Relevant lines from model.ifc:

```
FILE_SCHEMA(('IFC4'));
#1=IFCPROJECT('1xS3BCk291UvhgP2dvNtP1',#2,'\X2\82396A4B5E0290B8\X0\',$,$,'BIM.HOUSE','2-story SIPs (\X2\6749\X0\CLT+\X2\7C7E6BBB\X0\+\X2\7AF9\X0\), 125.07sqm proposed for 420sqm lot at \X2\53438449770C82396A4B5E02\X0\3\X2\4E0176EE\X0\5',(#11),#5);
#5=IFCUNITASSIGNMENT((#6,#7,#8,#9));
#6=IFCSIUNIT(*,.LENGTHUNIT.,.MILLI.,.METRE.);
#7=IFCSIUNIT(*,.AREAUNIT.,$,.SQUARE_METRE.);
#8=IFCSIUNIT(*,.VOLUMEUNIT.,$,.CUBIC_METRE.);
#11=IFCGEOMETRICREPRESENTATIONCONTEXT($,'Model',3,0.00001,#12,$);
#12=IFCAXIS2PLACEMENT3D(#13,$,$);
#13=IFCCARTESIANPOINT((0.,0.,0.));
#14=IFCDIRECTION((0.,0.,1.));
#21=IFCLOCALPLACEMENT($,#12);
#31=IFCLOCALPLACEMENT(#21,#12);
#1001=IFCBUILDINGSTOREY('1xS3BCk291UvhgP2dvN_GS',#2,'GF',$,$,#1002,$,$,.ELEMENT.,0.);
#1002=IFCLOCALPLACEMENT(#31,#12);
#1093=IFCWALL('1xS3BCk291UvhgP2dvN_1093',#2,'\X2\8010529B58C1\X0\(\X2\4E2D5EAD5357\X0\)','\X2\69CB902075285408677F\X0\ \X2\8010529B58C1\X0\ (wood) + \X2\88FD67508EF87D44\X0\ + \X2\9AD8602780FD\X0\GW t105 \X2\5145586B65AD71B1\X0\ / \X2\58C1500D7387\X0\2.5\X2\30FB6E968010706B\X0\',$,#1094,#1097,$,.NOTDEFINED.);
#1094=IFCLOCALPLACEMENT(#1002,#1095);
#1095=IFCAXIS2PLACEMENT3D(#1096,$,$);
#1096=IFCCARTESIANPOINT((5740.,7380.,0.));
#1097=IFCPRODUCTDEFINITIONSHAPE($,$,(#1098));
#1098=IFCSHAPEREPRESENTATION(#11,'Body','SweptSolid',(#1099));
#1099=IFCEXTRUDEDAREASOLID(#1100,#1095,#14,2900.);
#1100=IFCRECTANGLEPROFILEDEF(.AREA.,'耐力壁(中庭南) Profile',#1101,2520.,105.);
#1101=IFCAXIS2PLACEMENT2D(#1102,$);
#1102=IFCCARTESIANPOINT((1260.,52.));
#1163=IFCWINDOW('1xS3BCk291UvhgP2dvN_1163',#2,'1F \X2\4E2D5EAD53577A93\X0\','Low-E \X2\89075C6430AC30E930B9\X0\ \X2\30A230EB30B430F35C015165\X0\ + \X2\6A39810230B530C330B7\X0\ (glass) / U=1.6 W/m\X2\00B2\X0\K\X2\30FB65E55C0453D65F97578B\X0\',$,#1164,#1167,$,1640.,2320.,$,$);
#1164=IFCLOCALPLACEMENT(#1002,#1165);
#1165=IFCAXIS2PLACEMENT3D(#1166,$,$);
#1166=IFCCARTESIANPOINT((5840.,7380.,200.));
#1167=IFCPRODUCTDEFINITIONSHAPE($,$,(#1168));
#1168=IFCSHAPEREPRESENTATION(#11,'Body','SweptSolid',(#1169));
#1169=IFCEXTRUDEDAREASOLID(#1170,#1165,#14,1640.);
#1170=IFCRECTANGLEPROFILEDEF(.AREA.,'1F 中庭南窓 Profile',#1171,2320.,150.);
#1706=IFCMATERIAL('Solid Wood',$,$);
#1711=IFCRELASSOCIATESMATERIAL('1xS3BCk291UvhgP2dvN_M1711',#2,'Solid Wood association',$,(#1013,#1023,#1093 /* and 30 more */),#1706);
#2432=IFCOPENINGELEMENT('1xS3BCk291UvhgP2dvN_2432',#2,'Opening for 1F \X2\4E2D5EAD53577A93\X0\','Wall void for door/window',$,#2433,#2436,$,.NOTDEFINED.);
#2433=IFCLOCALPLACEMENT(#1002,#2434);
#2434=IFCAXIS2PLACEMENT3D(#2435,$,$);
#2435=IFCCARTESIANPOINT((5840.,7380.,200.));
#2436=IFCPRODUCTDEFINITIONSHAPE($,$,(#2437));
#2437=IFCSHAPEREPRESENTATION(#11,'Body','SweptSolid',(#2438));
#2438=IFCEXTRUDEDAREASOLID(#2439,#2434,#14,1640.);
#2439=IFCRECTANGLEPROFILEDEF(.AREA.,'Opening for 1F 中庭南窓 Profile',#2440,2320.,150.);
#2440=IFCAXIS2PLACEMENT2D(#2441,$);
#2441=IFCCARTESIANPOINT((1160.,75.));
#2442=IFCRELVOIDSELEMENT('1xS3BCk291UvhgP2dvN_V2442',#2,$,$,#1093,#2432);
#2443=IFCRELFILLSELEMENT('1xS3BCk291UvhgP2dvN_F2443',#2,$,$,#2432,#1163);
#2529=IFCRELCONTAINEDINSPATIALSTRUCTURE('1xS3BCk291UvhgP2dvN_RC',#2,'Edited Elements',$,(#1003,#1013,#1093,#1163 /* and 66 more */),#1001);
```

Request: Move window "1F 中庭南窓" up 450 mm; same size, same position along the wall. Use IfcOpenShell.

```python
import numpy as np
import ifcopenshell
import ifcopenshell.api.geometry
import ifcopenshell.util.placement
import ifcopenshell.util.unit

model = ifcopenshell.open("model.ifc")
unit_scale = ifcopenshell.util.unit.calculate_unit_scale(model)

window = model.by_guid("1xS3BCk291UvhgP2dvN_1163")
opening = window.FillsVoids[0].RelatingOpeningElement
dz = 0.45 / unit_scale

shift = np.array([0.0, 0.0, dz])
# The window is not placed relative to its opening, so move both.
for product in (opening, window):
    matrix = ifcopenshell.util.placement.get_local_placement(product.ObjectPlacement)
    matrix[:3, 3] += shift
    ifcopenshell.api.geometry.edit_object_placement(model, product=product, matrix=matrix, is_si=False)

print(f"moved by {dz * unit_scale:+.3f} m")

model.write("model-out.ifc")
```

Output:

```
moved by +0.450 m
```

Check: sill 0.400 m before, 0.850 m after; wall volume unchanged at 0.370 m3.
